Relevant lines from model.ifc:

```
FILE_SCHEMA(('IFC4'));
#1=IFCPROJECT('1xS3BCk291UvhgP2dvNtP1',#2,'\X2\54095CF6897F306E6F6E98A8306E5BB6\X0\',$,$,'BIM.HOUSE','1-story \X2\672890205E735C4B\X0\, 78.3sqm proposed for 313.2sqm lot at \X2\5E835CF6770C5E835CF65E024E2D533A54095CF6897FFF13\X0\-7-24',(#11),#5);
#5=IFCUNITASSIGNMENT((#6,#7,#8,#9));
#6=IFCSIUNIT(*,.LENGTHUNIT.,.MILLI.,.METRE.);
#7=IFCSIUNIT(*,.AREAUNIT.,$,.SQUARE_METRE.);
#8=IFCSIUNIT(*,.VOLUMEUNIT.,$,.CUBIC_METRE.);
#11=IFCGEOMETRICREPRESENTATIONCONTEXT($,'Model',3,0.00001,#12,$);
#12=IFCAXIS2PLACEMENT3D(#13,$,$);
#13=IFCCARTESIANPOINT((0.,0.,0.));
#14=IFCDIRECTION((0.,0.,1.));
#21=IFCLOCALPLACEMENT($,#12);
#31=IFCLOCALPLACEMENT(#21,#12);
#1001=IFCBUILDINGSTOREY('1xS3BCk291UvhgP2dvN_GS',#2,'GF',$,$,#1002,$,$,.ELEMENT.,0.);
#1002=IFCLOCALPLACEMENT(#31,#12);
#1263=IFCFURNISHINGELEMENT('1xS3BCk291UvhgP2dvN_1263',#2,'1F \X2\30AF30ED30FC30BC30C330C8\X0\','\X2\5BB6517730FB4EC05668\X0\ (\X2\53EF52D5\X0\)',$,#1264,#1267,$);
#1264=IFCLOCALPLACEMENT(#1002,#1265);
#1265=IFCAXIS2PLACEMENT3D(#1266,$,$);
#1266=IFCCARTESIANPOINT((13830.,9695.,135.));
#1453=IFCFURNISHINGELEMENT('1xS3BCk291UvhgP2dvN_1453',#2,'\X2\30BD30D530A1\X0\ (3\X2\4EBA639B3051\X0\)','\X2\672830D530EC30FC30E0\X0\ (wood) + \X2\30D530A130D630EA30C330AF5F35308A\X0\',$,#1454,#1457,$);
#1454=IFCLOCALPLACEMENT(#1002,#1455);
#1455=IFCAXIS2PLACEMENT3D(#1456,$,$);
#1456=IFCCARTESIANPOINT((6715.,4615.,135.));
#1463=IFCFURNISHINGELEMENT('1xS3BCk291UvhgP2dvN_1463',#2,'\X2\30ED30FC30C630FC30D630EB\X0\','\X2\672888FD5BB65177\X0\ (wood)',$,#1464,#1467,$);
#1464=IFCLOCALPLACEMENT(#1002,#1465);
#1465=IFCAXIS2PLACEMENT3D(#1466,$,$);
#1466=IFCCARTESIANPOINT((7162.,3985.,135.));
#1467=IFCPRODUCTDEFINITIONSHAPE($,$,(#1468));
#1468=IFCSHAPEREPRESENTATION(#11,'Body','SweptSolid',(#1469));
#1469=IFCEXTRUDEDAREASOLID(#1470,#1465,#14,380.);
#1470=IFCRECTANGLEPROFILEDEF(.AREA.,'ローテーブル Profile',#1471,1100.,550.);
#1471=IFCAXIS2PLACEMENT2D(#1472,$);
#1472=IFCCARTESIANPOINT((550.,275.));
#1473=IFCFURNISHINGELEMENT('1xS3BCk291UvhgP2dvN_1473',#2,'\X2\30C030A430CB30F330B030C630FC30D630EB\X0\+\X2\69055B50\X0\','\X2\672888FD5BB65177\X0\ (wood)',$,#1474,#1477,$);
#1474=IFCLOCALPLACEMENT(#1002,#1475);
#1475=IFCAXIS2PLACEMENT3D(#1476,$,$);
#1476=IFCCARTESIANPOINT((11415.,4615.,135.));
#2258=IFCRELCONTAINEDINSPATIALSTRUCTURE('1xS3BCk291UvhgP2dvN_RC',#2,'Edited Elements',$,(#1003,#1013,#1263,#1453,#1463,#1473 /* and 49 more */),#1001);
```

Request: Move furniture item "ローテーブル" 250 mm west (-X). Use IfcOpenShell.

```python
import ifcopenshell
import ifcopenshell.api.geometry
import ifcopenshell.util.placement
import ifcopenshell.util.unit

model = ifcopenshell.open("model.ifc")
unit_scale = ifcopenshell.util.unit.calculate_unit_scale(model)

item = model.by_id(1463)
matrix = ifcopenshell.util.placement.get_local_placement(item.ObjectPlacement)
matrix[0, 3] -= 0.25 / unit_scale
ifcopenshell.api.geometry.edit_object_placement(model, product=item, matrix=matrix, is_si=False)

print(ifcopenshell.util.placement.get_local_placement(item.ObjectPlacement).round(3) + 0.0)

model.write("model_updated.ifc")
```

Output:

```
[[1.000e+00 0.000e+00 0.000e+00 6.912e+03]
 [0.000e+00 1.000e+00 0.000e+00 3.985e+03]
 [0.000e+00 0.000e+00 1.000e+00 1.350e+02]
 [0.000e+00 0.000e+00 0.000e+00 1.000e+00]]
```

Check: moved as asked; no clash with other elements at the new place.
